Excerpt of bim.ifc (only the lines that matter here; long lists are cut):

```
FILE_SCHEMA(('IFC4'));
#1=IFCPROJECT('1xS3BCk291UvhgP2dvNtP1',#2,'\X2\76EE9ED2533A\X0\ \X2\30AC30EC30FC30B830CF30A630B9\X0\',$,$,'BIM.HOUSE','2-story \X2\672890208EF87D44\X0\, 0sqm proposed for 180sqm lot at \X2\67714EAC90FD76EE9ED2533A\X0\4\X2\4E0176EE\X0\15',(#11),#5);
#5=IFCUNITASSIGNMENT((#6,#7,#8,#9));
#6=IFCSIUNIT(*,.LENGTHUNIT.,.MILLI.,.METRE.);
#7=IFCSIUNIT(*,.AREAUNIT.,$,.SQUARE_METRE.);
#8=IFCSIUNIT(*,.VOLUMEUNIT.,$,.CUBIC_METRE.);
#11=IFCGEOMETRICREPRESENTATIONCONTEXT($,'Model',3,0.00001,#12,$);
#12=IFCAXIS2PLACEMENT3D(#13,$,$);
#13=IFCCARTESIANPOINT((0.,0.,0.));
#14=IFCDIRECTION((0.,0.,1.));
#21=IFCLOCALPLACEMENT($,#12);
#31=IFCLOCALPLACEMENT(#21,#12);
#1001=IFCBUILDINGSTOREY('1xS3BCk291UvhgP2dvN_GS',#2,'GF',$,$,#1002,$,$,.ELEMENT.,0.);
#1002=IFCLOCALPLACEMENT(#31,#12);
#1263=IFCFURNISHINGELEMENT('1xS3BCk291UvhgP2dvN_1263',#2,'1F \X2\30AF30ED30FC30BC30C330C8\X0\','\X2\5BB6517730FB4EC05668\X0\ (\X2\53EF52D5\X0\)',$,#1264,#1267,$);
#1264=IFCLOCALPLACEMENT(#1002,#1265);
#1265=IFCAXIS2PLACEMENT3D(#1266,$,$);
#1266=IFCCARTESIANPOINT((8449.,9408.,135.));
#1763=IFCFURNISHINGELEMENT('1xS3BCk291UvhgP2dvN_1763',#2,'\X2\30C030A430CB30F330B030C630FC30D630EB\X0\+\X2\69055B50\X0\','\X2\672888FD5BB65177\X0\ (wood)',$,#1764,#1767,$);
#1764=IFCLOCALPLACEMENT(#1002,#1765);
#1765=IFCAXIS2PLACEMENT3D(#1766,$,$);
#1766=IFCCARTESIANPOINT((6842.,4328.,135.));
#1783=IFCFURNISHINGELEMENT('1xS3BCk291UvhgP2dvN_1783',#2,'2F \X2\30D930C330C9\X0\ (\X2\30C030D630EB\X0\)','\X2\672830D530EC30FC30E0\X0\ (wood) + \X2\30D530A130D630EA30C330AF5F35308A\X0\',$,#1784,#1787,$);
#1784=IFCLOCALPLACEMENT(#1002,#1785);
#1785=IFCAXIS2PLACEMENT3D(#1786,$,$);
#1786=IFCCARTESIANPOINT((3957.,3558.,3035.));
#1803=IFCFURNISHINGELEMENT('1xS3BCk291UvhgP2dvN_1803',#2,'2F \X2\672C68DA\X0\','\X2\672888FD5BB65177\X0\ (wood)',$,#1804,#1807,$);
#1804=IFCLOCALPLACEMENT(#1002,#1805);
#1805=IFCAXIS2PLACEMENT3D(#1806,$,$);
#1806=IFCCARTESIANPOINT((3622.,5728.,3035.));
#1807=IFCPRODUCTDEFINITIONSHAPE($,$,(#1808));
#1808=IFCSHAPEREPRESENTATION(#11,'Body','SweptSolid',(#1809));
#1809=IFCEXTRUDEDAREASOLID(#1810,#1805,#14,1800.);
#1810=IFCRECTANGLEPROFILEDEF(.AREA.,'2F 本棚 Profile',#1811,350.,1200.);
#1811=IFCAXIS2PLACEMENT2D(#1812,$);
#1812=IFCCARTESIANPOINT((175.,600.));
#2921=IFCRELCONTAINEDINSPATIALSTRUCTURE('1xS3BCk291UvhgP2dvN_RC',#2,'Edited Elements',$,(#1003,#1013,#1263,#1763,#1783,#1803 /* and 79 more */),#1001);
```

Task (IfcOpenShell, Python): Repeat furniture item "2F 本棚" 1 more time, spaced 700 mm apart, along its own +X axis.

```python
import ifcopenshell
import ifcopenshell.api.geometry
import ifcopenshell.api.root
import ifcopenshell.util.element
import ifcopenshell.util.placement
import ifcopenshell.util.unit

model = ifcopenshell.open("bim.ifc")
unit_scale = ifcopenshell.util.unit.calculate_unit_scale(model)


def reuse_history(source, copy):
    """copy_class also copies each property set's owner history, people and application; keep the originals."""
    for rel in copy.IsDefinedBy:
        if rel.is_a("IfcRelDefinesByProperties") and (history := rel.RelatingPropertyDefinition.OwnerHistory):
            rel.RelatingPropertyDefinition.OwnerHistory = source.OwnerHistory
            ifcopenshell.util.element.remove_deep2(model, history)


source = model.by_guid("1xS3BCk291UvhgP2dvN_1803")
base = ifcopenshell.util.placement.get_local_placement(source.ObjectPlacement)
step = base[:3, 0] * 0.7 / unit_scale

for i in range(1, 2):
    copy = ifcopenshell.api.root.copy_class(model, product=source)
    copy.Representation = ifcopenshell.util.element.copy_deep(
        model, source.Representation, exclude=["IfcGeometricRepresentationContext", "IfcRepresentationMap"]
    )
    reuse_history(source, copy)
    matrix = base.copy()
    matrix[:3, 3] += i * step
    print("added at", matrix[:3, 3].round(3) + 0.0)
    ifcopenshell.api.geometry.edit_object_placement(model, product=copy, matrix=matrix, is_si=False)

model.write("bim_edited.ifc")
```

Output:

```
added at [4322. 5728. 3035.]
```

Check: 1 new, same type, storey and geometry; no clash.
